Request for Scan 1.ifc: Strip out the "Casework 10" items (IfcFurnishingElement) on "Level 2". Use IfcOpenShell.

First a look at what the model holds.

```python
import ifcopenshell
import ifcopenshell.util.element

model = ifcopenshell.open("Scan 1.ifc")
print(model.schema)
storey = next(s for s in model.by_type("IfcBuildingStorey") if s.Name == "Level 2")
furniture = [e for e in ifcopenshell.util.element.get_decomposition(storey) if e.is_a("IfcFurnishingElement")]
seen = {}
for e in furniture:
    element_type = ifcopenshell.util.element.get_type(e)
    name = element_type.Name if element_type not in (None, e) else None
    seen[name] = seen.get(name, 0) + 1
for name, count in sorted(seen.items(), key=str):
    print(count, "x", name)
```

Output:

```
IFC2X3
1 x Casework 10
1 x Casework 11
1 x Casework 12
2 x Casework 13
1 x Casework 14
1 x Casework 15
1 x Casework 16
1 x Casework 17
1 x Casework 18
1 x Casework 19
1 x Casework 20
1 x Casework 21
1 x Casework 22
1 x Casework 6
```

```python
import ifcopenshell
import ifcopenshell.api.root
import ifcopenshell.util.element

model = ifcopenshell.open("Scan 1.ifc")

storey = next(s for s in model.by_type("IfcBuildingStorey") if s.Name == "Level 2")
furniture = [e for e in ifcopenshell.util.element.get_decomposition(storey) if e.is_a("IfcFurnishingElement")]
targets = [e for e in furniture if (t := ifcopenshell.util.element.get_type(e)) not in (None, e) and t.Name == "Casework 10"]

for e in targets:
    ifcopenshell.api.root.remove_product(model, product=e)
print(len(targets), "removed")

model.write("Scan 1_edited.ifc")
```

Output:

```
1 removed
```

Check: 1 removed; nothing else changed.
